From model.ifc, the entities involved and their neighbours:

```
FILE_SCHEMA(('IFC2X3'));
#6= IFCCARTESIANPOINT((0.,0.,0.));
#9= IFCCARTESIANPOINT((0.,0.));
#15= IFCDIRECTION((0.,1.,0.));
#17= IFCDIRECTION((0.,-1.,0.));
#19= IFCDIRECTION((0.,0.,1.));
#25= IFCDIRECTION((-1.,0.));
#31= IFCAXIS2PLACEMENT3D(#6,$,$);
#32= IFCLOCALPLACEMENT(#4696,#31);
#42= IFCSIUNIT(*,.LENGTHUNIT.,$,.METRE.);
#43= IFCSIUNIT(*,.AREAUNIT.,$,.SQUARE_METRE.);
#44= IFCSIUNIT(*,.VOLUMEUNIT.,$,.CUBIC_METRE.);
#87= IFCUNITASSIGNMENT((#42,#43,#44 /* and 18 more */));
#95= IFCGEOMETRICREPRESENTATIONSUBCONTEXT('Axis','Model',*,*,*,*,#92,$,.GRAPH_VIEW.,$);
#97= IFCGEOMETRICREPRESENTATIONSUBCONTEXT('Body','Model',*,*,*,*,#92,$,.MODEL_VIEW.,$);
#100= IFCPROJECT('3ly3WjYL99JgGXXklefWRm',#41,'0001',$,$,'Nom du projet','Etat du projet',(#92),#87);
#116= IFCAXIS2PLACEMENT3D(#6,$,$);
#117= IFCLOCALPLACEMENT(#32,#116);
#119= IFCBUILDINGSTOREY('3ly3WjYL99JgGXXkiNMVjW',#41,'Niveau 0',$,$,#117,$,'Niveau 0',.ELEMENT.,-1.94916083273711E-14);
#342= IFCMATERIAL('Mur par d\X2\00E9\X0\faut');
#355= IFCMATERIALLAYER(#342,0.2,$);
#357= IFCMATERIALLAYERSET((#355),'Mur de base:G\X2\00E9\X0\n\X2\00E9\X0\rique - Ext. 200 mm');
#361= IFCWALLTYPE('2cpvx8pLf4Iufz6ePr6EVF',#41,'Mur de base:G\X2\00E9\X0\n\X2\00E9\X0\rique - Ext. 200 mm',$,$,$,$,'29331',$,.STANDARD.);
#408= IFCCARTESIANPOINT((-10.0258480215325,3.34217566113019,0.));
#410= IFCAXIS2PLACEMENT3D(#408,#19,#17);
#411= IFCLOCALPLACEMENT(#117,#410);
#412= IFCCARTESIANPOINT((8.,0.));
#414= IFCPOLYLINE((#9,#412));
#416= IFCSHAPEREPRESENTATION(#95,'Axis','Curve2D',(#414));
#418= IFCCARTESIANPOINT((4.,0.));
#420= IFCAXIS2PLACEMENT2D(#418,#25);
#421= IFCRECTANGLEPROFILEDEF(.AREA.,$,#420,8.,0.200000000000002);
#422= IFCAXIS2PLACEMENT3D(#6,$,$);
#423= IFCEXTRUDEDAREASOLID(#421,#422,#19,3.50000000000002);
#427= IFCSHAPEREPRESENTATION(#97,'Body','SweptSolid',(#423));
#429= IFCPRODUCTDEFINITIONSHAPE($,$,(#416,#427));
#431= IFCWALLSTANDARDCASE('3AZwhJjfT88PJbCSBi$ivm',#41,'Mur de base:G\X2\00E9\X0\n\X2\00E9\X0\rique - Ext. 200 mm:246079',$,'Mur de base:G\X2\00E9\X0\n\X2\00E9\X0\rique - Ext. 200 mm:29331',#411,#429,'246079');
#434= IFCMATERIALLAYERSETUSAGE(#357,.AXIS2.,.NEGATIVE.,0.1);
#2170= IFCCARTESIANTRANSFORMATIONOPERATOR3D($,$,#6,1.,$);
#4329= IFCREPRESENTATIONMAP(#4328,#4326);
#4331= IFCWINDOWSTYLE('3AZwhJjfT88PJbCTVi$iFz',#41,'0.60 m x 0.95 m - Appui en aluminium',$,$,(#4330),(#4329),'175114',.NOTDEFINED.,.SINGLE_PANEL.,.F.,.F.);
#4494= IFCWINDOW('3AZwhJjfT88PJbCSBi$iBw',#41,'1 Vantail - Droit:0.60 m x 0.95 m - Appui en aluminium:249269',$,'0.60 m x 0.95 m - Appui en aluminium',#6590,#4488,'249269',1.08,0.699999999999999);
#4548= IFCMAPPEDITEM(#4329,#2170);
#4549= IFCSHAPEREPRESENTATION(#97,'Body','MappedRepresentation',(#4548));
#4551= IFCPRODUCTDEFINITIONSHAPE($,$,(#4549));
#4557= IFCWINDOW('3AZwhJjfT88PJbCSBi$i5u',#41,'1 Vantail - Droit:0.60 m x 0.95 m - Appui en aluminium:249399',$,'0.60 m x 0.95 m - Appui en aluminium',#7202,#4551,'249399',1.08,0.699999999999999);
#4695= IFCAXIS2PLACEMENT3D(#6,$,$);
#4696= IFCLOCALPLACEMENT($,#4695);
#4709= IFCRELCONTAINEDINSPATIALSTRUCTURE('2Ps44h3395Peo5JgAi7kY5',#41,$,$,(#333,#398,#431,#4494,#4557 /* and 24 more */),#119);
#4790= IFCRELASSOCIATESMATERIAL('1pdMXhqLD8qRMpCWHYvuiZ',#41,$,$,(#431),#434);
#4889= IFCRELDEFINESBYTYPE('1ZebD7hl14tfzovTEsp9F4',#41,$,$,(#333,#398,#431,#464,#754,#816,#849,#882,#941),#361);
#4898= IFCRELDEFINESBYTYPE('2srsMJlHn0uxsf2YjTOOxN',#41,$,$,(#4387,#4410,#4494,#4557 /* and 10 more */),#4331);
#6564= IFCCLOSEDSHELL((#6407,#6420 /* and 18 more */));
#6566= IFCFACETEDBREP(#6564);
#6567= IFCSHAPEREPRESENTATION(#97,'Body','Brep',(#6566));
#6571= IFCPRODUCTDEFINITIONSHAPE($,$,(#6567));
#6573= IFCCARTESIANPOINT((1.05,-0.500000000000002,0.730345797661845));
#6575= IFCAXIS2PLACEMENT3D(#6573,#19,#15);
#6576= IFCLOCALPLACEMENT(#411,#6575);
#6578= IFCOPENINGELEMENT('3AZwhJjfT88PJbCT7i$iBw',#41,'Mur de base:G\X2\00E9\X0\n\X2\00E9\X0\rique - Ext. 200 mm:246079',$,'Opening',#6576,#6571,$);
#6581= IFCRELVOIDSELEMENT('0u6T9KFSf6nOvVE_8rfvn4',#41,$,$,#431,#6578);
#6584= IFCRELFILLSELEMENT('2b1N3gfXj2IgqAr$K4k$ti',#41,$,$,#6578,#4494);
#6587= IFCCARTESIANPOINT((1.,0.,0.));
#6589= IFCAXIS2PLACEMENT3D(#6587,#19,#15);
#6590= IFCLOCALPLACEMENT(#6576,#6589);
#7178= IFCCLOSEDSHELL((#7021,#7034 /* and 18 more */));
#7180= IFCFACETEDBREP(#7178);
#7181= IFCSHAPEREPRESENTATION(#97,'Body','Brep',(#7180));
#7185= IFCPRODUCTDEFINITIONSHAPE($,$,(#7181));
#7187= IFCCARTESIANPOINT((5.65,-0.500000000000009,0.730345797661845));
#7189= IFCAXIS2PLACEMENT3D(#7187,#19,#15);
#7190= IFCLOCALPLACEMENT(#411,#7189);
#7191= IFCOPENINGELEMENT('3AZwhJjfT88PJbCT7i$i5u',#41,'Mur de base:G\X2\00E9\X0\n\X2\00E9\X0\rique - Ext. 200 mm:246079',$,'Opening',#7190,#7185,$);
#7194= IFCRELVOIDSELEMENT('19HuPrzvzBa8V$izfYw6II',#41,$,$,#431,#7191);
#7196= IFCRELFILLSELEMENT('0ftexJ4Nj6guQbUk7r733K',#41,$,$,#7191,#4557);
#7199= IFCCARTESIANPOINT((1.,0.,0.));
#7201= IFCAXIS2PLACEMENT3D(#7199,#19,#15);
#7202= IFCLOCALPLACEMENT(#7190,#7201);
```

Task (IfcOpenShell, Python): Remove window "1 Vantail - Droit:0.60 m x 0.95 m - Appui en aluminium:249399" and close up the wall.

```python
import ifcopenshell
import ifcopenshell.api.feature
import ifcopenshell.api.root
import ifcopenshell.geom
import ifcopenshell.util.shape

model = ifcopenshell.open("model.ifc")
settings = ifcopenshell.geom.settings()


def volume(element):
    """Net volume in cubic metres, openings subtracted."""
    shape = ifcopenshell.geom.create_shape(settings, element)
    return ifcopenshell.util.shape.get_volume(shape.geometry)


window = model.by_guid("3AZwhJjfT88PJbCSBi$i5u")
opening = window.FillsVoids[0].RelatingOpeningElement
wall = opening.VoidsElements[0].RelatingBuildingElement
before = volume(wall)

ifcopenshell.api.root.remove_product(model, product=window)
ifcopenshell.api.feature.remove_feature(model, feature=opening)

after = volume(wall)

print(f"wall volume {before:.3f} -> {after:.3f} m3")

model.write("model_v2.ifc")
```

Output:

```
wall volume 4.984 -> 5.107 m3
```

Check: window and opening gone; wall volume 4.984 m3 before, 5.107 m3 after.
